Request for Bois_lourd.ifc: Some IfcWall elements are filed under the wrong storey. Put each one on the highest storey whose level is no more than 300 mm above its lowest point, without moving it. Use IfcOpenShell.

First a look at what the model holds.

```python
import ifcopenshell
import ifcopenshell.util.element
import ifcopenshell.util.placement

model = ifcopenshell.open("Bois_lourd.ifc")
print(model.schema)
for storey in model.by_type("IfcBuildingStorey"):
    level = ifcopenshell.util.placement.get_storey_elevation(storey)
    count = sum(e.is_a("IfcWall") for e in ifcopenshell.util.element.get_contained(storey))
    print(storey.id(), storey.Name, round(level, 3), count, sep=" | ")
```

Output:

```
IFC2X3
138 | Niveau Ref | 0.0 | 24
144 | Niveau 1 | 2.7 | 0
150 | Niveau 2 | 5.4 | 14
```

```python
import ifcopenshell
import ifcopenshell.api.spatial
import ifcopenshell.geom
import ifcopenshell.util.element
import ifcopenshell.util.placement
import ifcopenshell.util.shape
import ifcopenshell.util.unit

model = ifcopenshell.open("Bois_lourd.ifc")
unit_scale = ifcopenshell.util.unit.calculate_unit_scale(model)
settings = ifcopenshell.geom.settings()

levels = sorted(
    ((ifcopenshell.util.placement.get_storey_elevation(s) * unit_scale, s) for s in model.by_type("IfcBuildingStorey")),
    key=lambda pair: pair[0],
)

for e in model.by_type("IfcWall"):
    current = e.ContainedInStructure[0].RelatingStructure if e.ContainedInStructure else None
    if current is None or not current.is_a("IfcBuildingStorey"):
        continue
    shape = ifcopenshell.geom.create_shape(settings, e)
    bottom = ifcopenshell.util.shape.get_shape_bottom_elevation(shape, shape.geometry)
    below = [s for level, s in levels if level <= bottom + 0.3]
    storey = below[-1] if below else levels[0][1]
    if storey != current:
        # assign_container keeps the world position.
        ifcopenshell.api.spatial.assign_container(model, products=[e], relating_structure=storey)
        print(e.id(), current.Name, "->", storey.Name)

model.write("Bois_lourd_rev.ifc")
```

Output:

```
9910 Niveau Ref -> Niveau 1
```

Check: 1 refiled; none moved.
